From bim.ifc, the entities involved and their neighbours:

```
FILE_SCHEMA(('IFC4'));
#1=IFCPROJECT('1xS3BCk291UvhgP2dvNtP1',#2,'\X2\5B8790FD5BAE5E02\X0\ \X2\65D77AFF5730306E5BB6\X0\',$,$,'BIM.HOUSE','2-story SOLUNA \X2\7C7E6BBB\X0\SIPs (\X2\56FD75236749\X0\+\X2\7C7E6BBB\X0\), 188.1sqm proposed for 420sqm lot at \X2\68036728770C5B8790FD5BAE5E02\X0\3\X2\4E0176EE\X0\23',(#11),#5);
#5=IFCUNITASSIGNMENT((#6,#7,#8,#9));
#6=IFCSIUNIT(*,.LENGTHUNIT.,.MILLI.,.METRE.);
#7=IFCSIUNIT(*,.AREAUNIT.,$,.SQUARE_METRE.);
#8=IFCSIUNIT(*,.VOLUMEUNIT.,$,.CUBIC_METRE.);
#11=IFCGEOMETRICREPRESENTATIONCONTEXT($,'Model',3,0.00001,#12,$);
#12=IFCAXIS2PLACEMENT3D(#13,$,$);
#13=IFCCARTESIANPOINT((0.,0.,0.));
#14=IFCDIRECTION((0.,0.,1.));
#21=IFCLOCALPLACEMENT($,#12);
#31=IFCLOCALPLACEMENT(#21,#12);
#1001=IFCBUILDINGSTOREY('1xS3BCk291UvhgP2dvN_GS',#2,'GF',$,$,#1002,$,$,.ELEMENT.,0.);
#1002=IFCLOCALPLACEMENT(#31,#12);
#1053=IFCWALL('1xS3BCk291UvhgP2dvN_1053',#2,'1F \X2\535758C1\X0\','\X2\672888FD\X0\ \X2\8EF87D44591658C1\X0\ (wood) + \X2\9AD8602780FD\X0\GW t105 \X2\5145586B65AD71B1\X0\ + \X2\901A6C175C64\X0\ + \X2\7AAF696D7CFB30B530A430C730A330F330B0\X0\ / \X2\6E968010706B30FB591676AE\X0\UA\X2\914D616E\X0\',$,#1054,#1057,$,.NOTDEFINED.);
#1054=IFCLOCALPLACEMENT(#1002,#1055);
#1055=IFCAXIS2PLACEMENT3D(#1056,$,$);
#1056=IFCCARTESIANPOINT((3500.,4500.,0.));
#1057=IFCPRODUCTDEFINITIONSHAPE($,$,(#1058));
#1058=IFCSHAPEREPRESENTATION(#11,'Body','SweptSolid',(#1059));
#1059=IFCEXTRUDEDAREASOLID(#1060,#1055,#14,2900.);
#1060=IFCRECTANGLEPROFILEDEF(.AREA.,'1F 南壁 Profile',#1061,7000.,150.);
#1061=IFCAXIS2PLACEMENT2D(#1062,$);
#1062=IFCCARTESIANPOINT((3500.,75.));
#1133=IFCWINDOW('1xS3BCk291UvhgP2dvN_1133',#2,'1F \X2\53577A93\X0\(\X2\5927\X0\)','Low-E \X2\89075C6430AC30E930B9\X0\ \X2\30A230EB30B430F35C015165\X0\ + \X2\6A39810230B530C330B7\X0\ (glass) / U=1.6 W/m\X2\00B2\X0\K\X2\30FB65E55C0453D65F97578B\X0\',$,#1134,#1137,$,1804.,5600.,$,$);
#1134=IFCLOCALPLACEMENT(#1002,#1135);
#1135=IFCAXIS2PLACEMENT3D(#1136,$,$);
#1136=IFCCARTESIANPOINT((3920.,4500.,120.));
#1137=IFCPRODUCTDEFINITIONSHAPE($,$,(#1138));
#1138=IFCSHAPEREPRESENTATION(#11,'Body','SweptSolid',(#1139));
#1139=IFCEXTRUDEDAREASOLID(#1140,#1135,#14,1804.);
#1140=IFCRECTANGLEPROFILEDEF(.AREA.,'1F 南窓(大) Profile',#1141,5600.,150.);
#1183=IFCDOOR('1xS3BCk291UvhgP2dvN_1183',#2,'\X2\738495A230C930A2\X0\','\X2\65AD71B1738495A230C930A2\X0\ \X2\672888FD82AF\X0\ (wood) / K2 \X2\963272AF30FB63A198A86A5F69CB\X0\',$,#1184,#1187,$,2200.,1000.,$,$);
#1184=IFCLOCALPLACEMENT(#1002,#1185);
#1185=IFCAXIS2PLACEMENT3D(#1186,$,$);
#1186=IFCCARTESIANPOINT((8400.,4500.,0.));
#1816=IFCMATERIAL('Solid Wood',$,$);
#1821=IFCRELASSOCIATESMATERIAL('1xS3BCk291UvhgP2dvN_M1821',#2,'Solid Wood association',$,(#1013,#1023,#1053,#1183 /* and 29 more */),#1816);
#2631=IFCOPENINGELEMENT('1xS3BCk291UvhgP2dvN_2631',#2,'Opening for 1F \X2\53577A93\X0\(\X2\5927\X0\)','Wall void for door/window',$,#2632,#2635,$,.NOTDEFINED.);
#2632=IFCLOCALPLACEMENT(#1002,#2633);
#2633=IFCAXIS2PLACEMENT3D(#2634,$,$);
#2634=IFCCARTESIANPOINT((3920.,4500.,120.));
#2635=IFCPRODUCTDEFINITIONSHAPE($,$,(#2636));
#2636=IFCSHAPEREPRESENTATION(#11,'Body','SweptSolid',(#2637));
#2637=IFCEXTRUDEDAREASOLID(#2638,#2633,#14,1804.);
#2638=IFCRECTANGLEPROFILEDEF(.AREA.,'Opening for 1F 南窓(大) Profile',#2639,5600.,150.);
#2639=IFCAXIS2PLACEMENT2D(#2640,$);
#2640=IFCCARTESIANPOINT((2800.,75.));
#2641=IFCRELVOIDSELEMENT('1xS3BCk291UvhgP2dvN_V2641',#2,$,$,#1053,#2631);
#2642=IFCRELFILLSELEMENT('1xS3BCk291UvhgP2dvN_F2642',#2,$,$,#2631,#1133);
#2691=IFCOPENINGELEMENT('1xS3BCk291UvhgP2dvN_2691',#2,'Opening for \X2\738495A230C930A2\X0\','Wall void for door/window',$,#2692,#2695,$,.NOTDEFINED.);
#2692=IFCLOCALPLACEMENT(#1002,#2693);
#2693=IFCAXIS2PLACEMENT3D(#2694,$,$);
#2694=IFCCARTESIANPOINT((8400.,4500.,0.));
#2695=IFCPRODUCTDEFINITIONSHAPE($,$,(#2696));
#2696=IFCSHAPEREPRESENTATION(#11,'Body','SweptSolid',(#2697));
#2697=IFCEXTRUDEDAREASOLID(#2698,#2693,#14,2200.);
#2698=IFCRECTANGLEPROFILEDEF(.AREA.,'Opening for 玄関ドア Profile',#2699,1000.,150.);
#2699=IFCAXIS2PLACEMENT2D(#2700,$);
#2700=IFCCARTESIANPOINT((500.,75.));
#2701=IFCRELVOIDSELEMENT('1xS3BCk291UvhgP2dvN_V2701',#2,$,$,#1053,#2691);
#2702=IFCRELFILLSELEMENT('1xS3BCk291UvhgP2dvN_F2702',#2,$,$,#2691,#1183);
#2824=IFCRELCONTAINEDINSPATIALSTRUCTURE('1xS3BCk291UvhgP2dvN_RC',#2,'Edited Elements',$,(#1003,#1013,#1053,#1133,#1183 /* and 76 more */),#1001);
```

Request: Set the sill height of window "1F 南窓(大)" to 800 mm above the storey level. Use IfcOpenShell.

```python
import numpy as np
import ifcopenshell
import ifcopenshell.api.geometry
import ifcopenshell.geom
import ifcopenshell.util.element
import ifcopenshell.util.placement
import ifcopenshell.util.shape
import ifcopenshell.util.unit

model = ifcopenshell.open("bim.ifc")
unit_scale = ifcopenshell.util.unit.calculate_unit_scale(model)

window = model.by_guid("1xS3BCk291UvhgP2dvN_1133")
opening = window.FillsVoids[0].RelatingOpeningElement
storey = ifcopenshell.util.element.get_container(window, ifc_class="IfcBuildingStorey")
level = ifcopenshell.util.placement.get_local_placement(storey.ObjectPlacement)[2, 3]

# The opening's origin need not be at the sill, so measure its lowest point.
shape = ifcopenshell.geom.create_shape(ifcopenshell.geom.settings(), opening)
bottom = ifcopenshell.util.shape.get_shape_bottom_elevation(shape, shape.geometry) / unit_scale
dz = level + 0.8 / unit_scale - bottom

shift = np.array([0.0, 0.0, dz])
# The window is not placed relative to its opening, so move both.
for product in (opening, window):
    matrix = ifcopenshell.util.placement.get_local_placement(product.ObjectPlacement)
    matrix[:3, 3] += shift
    ifcopenshell.api.geometry.edit_object_placement(model, product=product, matrix=matrix, is_si=False)

print(f"moved by {dz * unit_scale:+.3f} m")

model.write("bim_rev.ifc")
```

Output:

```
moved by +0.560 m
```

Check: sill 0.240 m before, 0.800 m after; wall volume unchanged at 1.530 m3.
